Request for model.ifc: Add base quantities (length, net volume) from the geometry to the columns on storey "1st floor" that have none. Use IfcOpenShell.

First a look at what the model holds.

```python
import ifcopenshell
import ifcopenshell.util.element
import ifcopenshell.util.unit

model = ifcopenshell.open("model.ifc")
print(model.schema)
for unit_type in ("LENGTHUNIT", "AREAUNIT", "VOLUMEUNIT"):
    print(unit_type, ifcopenshell.util.unit.calculate_unit_scale(model, unit_type))
storey = next(s for s in model.by_type("IfcBuildingStorey") if s.Name == "1st floor")
columns = [e for e in ifcopenshell.util.element.get_decomposition(storey) if e.is_a("IfcColumn")]
for e in sorted(columns, key=lambda e: e.id()):
    print(e.id(), e.is_a(), e.Name, list(ifcopenshell.util.element.get_psets(e, qtos_only=True)), sep=" | ")
```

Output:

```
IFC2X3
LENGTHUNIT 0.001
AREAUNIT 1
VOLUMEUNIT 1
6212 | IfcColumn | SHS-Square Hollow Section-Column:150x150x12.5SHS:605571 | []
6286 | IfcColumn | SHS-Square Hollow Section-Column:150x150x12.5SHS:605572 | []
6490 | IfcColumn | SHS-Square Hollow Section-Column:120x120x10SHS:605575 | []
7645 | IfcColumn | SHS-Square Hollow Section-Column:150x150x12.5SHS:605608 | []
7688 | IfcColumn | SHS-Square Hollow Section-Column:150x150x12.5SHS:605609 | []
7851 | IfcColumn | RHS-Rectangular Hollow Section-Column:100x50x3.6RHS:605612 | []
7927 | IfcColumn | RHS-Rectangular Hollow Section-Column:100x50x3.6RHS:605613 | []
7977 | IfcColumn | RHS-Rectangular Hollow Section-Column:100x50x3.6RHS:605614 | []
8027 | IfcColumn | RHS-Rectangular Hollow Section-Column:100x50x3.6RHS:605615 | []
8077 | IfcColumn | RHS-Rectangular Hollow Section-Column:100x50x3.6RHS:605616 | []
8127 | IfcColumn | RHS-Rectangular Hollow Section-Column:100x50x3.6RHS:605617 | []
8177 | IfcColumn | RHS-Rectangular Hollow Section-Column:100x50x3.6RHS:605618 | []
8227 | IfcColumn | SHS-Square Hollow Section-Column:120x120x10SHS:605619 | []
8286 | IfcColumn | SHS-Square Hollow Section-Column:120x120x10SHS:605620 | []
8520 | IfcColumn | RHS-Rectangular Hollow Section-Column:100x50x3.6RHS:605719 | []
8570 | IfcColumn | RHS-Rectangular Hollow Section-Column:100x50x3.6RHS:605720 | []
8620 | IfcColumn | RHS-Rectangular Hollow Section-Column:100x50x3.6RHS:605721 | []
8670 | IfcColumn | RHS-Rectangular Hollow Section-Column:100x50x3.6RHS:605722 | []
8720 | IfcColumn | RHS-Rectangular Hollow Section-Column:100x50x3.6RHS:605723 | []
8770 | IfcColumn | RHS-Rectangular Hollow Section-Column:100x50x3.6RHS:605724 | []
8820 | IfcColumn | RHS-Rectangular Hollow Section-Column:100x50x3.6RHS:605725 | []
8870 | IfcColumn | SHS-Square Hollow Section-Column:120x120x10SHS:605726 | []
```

```python
import ifcopenshell
import ifcopenshell.api.pset
import ifcopenshell.geom
import ifcopenshell.util.element
import ifcopenshell.util.shape
import ifcopenshell.util.unit

model = ifcopenshell.open("model.ifc")
unit_scale = ifcopenshell.util.unit.calculate_unit_scale(model)
volume_scale = ifcopenshell.util.unit.calculate_unit_scale(model, "VOLUMEUNIT")
settings = ifcopenshell.geom.settings()

storey = next(s for s in model.by_type("IfcBuildingStorey") if s.Name == "1st floor")
columns = [e for e in ifcopenshell.util.element.get_decomposition(storey) if e.is_a("IfcColumn")]

for e in sorted(columns, key=lambda e: e.id()):
    if ifcopenshell.util.element.get_psets(e, qtos_only=True, should_inherit=False):
        continue
    # Geometry comes back in metres, in the element's own axes.
    shape = ifcopenshell.geom.create_shape(settings, e)
    values = {
        "Length": ifcopenshell.util.shape.get_z(shape.geometry) / unit_scale,
        "NetVolume": ifcopenshell.util.shape.get_volume(shape.geometry) / volume_scale,
    }
    qto = ifcopenshell.api.pset.add_qto(model, product=e, name="BaseQuantities")
    ifcopenshell.api.pset.edit_qto(model, qto=qto, properties=values)
    print(e.id(), {k: round(v, 3) for k, v in values.items()})

model.write("model_rev.ifc")
```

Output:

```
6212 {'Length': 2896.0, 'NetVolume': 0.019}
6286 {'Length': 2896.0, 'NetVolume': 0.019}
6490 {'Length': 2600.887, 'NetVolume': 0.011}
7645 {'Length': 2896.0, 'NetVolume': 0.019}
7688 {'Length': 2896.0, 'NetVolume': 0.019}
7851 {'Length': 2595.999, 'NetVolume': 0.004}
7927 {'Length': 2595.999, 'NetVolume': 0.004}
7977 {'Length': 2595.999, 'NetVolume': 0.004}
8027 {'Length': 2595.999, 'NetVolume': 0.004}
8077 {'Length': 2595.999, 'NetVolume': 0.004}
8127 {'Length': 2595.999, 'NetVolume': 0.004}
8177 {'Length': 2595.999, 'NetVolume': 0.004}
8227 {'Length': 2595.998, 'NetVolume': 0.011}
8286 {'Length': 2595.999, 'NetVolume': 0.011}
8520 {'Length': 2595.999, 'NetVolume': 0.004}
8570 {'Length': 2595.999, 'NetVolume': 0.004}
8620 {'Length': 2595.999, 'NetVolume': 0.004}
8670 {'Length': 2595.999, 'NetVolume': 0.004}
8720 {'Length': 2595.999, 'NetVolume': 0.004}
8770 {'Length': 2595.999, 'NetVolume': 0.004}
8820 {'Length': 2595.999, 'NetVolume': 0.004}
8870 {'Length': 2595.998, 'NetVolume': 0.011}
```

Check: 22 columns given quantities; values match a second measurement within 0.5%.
